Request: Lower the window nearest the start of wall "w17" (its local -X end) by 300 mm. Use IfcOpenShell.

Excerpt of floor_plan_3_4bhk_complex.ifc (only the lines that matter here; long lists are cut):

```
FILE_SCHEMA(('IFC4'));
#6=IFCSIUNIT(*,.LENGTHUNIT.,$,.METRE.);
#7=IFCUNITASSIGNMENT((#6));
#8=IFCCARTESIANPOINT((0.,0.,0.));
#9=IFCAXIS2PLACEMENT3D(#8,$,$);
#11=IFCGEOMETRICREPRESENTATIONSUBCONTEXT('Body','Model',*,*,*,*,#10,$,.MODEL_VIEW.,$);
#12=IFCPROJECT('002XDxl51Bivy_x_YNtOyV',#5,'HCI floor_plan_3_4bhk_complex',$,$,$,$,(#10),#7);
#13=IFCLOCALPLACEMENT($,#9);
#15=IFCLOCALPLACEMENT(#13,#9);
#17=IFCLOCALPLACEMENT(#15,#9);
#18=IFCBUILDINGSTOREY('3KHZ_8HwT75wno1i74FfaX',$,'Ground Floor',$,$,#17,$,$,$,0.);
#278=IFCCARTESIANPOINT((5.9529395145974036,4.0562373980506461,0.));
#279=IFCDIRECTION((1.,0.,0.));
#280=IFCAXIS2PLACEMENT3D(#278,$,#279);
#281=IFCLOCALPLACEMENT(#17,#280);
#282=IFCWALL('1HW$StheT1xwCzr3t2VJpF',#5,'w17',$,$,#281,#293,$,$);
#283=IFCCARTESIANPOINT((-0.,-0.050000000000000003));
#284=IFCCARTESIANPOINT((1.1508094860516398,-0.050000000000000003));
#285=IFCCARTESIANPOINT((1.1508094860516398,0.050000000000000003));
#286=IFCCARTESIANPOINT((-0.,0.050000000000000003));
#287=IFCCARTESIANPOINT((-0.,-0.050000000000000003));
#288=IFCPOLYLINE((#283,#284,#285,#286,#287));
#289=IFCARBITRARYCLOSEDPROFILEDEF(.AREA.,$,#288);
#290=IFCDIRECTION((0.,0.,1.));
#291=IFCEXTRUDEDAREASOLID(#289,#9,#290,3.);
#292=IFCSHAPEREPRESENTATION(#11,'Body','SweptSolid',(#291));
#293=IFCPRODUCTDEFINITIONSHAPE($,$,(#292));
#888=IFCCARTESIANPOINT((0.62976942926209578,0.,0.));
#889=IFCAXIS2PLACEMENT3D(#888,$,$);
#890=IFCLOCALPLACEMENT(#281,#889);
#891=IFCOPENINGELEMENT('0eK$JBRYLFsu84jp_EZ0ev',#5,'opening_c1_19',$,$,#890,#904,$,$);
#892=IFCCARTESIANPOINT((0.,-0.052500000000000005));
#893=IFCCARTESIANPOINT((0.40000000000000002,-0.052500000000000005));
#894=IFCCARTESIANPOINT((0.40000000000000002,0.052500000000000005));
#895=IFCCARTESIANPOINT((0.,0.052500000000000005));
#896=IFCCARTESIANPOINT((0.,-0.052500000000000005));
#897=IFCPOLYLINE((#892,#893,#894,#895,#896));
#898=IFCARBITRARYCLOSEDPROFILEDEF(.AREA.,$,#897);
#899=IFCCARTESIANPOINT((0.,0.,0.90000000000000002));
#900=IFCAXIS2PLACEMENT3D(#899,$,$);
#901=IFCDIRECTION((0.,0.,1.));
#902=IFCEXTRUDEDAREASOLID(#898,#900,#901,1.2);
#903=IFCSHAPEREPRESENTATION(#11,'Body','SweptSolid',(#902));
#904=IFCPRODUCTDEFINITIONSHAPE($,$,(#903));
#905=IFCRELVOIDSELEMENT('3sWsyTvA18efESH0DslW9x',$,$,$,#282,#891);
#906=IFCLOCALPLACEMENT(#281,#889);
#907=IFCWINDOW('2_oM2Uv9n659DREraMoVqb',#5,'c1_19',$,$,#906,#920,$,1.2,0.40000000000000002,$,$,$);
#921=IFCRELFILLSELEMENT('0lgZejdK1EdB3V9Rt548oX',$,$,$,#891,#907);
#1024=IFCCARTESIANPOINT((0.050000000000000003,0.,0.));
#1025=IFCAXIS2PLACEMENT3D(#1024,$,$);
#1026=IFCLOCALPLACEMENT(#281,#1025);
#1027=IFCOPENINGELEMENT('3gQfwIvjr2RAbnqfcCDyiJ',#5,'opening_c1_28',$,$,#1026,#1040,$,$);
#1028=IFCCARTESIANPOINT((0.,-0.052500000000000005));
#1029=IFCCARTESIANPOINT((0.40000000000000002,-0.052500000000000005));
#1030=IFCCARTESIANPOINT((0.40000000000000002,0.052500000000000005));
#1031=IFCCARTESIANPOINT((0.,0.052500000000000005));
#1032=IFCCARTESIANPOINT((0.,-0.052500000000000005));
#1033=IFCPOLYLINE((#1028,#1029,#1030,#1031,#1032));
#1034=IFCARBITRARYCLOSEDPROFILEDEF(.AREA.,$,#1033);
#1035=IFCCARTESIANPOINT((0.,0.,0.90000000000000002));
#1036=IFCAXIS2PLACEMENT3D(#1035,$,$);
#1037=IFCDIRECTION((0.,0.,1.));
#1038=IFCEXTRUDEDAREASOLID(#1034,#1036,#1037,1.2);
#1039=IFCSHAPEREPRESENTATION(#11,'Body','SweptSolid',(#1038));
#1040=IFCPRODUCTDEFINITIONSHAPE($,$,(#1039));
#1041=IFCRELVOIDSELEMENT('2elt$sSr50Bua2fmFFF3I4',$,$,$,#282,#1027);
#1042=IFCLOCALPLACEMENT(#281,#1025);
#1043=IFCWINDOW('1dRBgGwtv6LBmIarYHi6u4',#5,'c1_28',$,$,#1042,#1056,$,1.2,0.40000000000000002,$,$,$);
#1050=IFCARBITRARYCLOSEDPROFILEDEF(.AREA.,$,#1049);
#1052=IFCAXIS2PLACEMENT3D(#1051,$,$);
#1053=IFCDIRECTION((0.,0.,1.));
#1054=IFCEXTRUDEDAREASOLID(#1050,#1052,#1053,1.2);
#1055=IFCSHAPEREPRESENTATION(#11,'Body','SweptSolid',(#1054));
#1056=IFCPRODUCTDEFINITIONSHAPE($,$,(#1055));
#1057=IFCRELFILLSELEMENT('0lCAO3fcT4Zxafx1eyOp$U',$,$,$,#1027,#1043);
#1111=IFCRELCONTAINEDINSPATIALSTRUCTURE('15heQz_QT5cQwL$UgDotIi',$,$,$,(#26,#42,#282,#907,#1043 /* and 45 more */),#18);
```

```python
import numpy as np
import ifcopenshell
import ifcopenshell.api.geometry
import ifcopenshell.util.placement
import ifcopenshell.util.unit

model = ifcopenshell.open("floor_plan_3_4bhk_complex.ifc")
unit_scale = ifcopenshell.util.unit.calculate_unit_scale(model)

window = model.by_id(1043)
opening = window.FillsVoids[0].RelatingOpeningElement
dz = -0.3

shift = np.array([0.0, 0.0, dz])
# The window is not placed relative to its opening, so move both.
for product in (opening, window):
    matrix = ifcopenshell.util.placement.get_local_placement(product.ObjectPlacement)
    matrix[:3, 3] += shift
    ifcopenshell.api.geometry.edit_object_placement(model, product=product, matrix=matrix, is_si=False)

print(f"moved by {dz * unit_scale:+.3f} m")

model.write("floor_plan_3_4bhk_complex_v2.ifc")
```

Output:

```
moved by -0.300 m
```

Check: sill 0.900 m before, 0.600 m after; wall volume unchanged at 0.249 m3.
